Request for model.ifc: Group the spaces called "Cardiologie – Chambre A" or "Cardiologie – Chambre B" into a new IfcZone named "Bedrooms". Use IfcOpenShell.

First a look at what the model holds.

```python
import ifcopenshell

model = ifcopenshell.open("model.ifc")
print(model.schema)
seen = {}
for space in model.by_type("IfcSpace"):
    seen[space.LongName] = seen.get(space.LongName, 0) + 1
for name, count in sorted(seen.items(), key=str):
    print(count, "x", name)
print("zones:", [z.Name for z in model.by_type("IfcZone")][:20])
```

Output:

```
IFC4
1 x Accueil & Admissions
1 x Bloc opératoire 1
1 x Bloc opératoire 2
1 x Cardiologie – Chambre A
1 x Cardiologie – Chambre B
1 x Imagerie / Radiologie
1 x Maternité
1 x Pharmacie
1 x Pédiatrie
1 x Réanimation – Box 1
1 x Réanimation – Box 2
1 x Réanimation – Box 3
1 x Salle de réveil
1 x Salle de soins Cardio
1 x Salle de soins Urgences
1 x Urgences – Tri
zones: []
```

```python
import ifcopenshell
import ifcopenshell.api.group
import ifcopenshell.api.root

model = ifcopenshell.open("model.ifc")

names = {"Cardiologie – Chambre A", "Cardiologie – Chambre B"}
spaces = [s for s in model.by_type("IfcSpace") if s.LongName in names]

zone = ifcopenshell.api.root.create_entity(model, ifc_class="IfcZone", name="Bedrooms")
ifcopenshell.api.group.assign_group(model, products=spaces, group=zone)
print(len(spaces), "spaces in", zone.Name)

model.write("model_v2.ifc")
```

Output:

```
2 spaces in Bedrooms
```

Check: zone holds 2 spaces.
